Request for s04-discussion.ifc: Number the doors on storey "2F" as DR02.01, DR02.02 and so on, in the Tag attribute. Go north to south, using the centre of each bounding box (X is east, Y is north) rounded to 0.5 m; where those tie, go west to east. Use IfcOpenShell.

First a look at what the model holds.

```python
import ifcopenshell
import ifcopenshell.util.element
import ifcopenshell.util.placement

model = ifcopenshell.open("s04-discussion.ifc")
print(model.schema)
storey = next(s for s in model.by_type("IfcBuildingStorey") if s.Name == "2F")
doors = [e for e in ifcopenshell.util.element.get_decomposition(storey) if e.is_a("IfcDoor")]
for e in sorted(doors, key=lambda e: e.id()):
    origin = ifcopenshell.util.placement.get_local_placement(e.ObjectPlacement)[:3, 3]
    print(e.id(), e.Tag, e.Name, origin.round(2) + 0.0, sep=" | ")
```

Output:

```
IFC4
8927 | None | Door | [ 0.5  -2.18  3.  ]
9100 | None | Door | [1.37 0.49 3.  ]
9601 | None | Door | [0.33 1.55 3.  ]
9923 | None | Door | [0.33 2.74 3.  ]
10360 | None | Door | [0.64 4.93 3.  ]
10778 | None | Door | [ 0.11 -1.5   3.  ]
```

```python
import ifcopenshell
import ifcopenshell.geom
import ifcopenshell.util.element
import ifcopenshell.util.shape

model = ifcopenshell.open("s04-discussion.ifc")
settings = ifcopenshell.geom.settings()
settings.set("use-world-coords", True)


def centre(element):
    shape = ifcopenshell.geom.create_shape(settings, element)
    return ifcopenshell.util.shape.get_bbox_centroid(shape.geometry)


storey = next(s for s in model.by_type("IfcBuildingStorey") if s.Name == "2F")
doors = [e for e in ifcopenshell.util.element.get_decomposition(storey) if e.is_a("IfcDoor")]

# Insertion points can sit at a corner or the storey origin, so sort by the geometry (in metres).
centres = {e: centre(e) for e in doors}
doors.sort(key=lambda e: (-round(centres[e][1] / 0.5), centres[e][0]))

for i, e in enumerate(doors, start=1):
    number = f"DR02.{i:02d}"
    e.Tag = number
    print(e.id(), number)

model.write("s04-discussion_v2.ifc")
```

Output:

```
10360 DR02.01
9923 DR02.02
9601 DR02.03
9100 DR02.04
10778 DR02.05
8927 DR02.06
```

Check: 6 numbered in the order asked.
